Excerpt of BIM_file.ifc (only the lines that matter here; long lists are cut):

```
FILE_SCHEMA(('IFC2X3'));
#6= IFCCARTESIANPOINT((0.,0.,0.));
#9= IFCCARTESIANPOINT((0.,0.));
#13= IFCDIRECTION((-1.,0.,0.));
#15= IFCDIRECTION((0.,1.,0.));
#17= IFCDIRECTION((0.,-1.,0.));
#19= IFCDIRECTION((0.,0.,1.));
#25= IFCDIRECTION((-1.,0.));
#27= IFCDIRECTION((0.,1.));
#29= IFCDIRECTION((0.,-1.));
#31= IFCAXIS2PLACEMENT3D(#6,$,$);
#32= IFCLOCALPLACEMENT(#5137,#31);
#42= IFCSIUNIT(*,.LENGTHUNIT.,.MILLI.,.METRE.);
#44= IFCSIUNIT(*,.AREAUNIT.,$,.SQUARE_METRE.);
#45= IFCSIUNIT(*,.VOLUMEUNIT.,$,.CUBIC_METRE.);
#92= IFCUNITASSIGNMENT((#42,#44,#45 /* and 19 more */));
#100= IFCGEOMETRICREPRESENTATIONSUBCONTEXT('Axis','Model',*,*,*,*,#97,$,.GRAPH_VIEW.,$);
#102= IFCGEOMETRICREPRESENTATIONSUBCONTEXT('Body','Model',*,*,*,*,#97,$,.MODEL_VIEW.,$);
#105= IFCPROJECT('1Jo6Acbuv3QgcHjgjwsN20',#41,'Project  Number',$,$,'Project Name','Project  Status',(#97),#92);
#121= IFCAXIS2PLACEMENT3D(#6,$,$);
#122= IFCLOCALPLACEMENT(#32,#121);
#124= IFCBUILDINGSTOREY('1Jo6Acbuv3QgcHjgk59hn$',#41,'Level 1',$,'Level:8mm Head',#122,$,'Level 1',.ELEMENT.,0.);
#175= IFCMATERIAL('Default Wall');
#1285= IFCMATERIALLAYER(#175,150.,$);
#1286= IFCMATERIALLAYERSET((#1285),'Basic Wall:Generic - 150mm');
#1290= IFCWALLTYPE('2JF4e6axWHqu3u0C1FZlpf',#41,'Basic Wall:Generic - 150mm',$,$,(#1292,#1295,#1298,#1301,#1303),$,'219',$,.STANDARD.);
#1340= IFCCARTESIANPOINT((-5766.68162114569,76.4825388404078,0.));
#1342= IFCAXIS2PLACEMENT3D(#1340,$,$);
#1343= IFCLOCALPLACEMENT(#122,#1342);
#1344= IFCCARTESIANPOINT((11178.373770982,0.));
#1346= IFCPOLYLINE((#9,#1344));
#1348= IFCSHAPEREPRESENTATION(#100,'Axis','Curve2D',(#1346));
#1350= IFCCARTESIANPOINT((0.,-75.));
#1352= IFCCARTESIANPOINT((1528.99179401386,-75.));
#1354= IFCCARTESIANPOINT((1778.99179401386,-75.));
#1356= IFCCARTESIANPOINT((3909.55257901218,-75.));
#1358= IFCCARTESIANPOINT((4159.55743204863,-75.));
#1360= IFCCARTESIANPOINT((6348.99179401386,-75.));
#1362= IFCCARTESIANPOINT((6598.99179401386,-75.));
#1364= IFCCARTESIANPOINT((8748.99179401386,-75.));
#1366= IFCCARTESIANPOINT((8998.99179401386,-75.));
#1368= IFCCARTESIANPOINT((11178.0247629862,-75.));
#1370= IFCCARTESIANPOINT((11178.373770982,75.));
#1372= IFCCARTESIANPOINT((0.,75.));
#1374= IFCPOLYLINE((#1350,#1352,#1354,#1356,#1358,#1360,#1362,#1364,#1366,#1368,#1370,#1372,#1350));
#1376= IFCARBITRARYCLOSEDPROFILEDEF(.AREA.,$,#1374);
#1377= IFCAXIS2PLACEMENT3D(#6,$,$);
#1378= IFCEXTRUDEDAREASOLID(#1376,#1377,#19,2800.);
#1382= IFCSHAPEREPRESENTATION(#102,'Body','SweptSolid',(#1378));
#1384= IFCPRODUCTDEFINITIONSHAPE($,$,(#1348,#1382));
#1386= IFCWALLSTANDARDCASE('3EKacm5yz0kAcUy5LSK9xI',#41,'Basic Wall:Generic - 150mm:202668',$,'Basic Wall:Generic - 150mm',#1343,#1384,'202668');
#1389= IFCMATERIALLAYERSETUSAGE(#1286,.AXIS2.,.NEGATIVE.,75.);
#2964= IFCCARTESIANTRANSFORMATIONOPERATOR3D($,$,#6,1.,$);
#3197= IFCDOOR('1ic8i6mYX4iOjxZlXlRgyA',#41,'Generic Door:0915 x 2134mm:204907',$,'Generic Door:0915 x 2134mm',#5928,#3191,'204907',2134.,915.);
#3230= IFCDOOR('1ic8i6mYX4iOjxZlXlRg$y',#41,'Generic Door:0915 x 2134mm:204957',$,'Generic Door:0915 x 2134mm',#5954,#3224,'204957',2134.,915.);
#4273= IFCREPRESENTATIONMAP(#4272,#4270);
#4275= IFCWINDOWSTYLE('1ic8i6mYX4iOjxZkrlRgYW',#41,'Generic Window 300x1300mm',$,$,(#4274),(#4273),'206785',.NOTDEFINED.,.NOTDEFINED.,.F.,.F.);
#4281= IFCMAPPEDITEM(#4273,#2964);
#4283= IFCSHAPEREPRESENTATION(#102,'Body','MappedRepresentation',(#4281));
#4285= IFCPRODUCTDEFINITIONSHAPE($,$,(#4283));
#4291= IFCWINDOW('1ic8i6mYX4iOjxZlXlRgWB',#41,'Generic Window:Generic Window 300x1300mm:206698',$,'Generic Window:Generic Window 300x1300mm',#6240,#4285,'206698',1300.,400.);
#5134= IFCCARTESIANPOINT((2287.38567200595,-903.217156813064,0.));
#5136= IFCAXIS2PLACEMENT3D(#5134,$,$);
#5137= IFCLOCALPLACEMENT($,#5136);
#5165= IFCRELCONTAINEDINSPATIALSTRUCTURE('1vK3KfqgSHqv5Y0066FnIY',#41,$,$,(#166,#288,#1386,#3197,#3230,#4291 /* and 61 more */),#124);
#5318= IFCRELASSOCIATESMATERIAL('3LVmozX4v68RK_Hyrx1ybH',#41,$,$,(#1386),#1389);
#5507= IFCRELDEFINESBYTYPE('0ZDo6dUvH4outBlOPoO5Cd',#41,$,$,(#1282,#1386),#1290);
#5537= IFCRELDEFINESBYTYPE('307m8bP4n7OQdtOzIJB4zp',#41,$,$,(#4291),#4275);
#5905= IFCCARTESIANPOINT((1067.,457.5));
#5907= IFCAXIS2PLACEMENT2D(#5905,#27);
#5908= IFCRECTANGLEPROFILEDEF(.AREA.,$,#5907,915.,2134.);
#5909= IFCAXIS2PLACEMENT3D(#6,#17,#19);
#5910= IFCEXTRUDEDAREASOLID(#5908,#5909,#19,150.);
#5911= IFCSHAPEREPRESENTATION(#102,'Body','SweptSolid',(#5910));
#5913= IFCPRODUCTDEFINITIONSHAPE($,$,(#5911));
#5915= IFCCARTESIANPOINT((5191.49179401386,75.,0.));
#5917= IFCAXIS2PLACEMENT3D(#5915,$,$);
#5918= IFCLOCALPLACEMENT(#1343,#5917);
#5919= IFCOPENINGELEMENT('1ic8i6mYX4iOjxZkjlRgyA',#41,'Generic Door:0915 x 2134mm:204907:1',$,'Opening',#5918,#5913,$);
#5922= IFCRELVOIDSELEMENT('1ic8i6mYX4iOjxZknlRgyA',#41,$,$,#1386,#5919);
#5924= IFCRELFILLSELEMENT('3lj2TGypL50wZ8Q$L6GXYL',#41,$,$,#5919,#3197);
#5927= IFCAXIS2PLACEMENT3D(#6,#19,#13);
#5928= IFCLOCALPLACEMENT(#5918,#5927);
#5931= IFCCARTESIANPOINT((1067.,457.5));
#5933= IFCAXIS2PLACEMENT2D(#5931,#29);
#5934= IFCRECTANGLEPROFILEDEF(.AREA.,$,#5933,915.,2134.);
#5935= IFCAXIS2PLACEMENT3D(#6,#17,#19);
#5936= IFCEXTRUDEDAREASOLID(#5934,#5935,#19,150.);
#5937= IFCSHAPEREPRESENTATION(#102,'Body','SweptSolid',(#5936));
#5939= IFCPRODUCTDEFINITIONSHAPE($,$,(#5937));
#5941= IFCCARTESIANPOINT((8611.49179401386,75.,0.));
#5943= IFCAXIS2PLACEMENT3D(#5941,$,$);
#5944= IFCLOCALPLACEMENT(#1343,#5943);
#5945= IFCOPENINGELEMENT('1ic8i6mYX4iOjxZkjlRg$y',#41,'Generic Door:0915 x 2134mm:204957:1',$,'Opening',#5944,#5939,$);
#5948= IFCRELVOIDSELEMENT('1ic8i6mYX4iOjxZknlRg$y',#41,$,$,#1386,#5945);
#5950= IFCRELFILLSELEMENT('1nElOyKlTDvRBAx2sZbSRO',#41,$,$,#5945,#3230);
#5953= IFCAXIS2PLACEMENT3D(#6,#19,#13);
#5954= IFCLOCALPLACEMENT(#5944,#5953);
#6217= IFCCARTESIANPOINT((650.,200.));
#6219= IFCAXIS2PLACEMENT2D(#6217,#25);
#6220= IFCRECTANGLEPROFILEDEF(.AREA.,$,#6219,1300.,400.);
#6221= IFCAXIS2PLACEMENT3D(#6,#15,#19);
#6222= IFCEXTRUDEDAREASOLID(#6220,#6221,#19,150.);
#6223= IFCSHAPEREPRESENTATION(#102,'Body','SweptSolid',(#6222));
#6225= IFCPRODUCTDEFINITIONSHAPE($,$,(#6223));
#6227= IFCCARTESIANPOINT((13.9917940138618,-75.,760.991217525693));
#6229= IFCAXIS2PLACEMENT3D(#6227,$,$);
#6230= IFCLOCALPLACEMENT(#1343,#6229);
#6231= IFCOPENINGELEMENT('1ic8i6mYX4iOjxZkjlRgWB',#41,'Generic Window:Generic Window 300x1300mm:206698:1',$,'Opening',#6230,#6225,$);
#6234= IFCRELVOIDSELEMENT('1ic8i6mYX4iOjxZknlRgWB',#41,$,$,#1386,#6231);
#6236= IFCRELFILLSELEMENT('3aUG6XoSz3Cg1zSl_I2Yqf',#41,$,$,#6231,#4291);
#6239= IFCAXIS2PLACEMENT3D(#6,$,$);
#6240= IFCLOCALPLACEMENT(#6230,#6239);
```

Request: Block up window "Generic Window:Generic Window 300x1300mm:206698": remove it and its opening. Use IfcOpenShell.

```python
import ifcopenshell
import ifcopenshell.api.feature
import ifcopenshell.api.root
import ifcopenshell.geom
import ifcopenshell.util.shape

model = ifcopenshell.open("BIM_file.ifc")
settings = ifcopenshell.geom.settings()


def volume(element):
    """Net volume in cubic metres, openings subtracted."""
    shape = ifcopenshell.geom.create_shape(settings, element)
    return ifcopenshell.util.shape.get_volume(shape.geometry)


window = model.by_id(4291)
opening = window.FillsVoids[0].RelatingOpeningElement
wall = opening.VoidsElements[0].RelatingBuildingElement
before = volume(wall)

ifcopenshell.api.root.remove_product(model, product=window)
ifcopenshell.api.feature.remove_feature(model, feature=opening)

after = volume(wall)

print(f"wall volume {before:.3f} -> {after:.3f} m3")

model.write("BIM_file_rev.ifc")
```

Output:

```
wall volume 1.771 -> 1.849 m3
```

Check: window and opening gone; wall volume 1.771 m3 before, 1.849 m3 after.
